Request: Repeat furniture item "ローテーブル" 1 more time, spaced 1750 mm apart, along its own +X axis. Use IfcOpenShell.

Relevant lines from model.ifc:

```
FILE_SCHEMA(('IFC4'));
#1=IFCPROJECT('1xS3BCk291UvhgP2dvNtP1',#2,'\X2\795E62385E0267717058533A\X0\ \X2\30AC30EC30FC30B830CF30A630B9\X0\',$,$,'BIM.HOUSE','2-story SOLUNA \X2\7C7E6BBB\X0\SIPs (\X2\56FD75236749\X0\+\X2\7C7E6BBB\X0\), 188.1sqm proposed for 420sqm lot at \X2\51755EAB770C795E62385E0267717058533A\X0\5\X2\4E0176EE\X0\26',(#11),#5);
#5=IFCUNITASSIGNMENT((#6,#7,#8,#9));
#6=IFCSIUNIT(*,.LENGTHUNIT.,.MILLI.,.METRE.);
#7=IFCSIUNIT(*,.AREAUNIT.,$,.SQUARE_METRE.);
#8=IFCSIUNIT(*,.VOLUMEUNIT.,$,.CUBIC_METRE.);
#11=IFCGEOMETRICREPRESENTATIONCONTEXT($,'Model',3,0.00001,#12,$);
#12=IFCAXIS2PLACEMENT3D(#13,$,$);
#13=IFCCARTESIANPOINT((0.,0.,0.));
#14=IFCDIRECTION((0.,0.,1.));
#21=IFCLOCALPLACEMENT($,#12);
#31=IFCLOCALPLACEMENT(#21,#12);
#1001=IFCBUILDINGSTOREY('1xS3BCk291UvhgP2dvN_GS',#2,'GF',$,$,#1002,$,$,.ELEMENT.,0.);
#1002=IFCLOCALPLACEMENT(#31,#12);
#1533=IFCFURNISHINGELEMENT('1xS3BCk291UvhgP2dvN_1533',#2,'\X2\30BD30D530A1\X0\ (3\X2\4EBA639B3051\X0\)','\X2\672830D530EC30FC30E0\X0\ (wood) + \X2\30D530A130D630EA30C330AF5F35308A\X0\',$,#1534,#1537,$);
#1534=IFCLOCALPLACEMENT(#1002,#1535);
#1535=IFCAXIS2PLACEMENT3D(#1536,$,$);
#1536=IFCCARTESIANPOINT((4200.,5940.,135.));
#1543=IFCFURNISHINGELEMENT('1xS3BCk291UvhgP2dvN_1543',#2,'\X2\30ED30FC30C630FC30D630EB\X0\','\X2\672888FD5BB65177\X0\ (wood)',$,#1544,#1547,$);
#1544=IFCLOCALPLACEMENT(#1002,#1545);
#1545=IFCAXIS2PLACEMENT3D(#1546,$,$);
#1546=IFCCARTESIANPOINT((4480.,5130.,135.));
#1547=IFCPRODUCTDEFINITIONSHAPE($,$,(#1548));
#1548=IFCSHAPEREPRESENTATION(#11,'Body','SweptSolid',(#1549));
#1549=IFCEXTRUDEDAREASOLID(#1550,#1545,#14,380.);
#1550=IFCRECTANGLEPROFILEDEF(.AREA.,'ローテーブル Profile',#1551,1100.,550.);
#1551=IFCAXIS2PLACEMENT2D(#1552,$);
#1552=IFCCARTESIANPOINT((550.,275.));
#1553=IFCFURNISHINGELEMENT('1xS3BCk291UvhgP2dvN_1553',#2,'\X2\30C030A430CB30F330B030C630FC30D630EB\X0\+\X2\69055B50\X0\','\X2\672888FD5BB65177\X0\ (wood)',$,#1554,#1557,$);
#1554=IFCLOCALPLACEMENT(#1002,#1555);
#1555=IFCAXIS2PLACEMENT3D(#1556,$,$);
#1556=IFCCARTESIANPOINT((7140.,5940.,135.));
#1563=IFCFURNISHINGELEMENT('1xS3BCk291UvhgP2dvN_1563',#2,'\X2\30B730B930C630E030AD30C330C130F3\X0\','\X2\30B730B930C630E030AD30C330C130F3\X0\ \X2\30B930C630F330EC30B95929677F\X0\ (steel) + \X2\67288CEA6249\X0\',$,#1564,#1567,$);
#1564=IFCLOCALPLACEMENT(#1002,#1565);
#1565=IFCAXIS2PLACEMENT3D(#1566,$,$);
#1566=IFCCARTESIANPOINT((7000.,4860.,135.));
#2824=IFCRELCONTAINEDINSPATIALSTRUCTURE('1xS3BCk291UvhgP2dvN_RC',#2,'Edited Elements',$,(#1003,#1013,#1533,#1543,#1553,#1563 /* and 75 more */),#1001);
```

```python
import ifcopenshell
import ifcopenshell.api.geometry
import ifcopenshell.api.root
import ifcopenshell.util.element
import ifcopenshell.util.placement
import ifcopenshell.util.unit

model = ifcopenshell.open("model.ifc")
unit_scale = ifcopenshell.util.unit.calculate_unit_scale(model)


def reuse_history(source, copy):
    """copy_class also copies each property set's owner history, people and application; keep the originals."""
    for rel in copy.IsDefinedBy:
        if rel.is_a("IfcRelDefinesByProperties") and (history := rel.RelatingPropertyDefinition.OwnerHistory):
            rel.RelatingPropertyDefinition.OwnerHistory = source.OwnerHistory
            ifcopenshell.util.element.remove_deep2(model, history)


source = model.by_guid("1xS3BCk291UvhgP2dvN_1543")
base = ifcopenshell.util.placement.get_local_placement(source.ObjectPlacement)
step = base[:3, 0] * 1.75 / unit_scale

for i in range(1, 2):
    copy = ifcopenshell.api.root.copy_class(model, product=source)
    copy.Representation = ifcopenshell.util.element.copy_deep(
        model, source.Representation, exclude=["IfcGeometricRepresentationContext", "IfcRepresentationMap"]
    )
    reuse_history(source, copy)
    matrix = base.copy()
    matrix[:3, 3] += i * step
    print("added at", matrix[:3, 3].round(3) + 0.0)
    ifcopenshell.api.geometry.edit_object_placement(model, product=copy, matrix=matrix, is_si=False)

model.write("model_edited.ifc")
```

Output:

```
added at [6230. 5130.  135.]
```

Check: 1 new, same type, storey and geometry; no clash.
